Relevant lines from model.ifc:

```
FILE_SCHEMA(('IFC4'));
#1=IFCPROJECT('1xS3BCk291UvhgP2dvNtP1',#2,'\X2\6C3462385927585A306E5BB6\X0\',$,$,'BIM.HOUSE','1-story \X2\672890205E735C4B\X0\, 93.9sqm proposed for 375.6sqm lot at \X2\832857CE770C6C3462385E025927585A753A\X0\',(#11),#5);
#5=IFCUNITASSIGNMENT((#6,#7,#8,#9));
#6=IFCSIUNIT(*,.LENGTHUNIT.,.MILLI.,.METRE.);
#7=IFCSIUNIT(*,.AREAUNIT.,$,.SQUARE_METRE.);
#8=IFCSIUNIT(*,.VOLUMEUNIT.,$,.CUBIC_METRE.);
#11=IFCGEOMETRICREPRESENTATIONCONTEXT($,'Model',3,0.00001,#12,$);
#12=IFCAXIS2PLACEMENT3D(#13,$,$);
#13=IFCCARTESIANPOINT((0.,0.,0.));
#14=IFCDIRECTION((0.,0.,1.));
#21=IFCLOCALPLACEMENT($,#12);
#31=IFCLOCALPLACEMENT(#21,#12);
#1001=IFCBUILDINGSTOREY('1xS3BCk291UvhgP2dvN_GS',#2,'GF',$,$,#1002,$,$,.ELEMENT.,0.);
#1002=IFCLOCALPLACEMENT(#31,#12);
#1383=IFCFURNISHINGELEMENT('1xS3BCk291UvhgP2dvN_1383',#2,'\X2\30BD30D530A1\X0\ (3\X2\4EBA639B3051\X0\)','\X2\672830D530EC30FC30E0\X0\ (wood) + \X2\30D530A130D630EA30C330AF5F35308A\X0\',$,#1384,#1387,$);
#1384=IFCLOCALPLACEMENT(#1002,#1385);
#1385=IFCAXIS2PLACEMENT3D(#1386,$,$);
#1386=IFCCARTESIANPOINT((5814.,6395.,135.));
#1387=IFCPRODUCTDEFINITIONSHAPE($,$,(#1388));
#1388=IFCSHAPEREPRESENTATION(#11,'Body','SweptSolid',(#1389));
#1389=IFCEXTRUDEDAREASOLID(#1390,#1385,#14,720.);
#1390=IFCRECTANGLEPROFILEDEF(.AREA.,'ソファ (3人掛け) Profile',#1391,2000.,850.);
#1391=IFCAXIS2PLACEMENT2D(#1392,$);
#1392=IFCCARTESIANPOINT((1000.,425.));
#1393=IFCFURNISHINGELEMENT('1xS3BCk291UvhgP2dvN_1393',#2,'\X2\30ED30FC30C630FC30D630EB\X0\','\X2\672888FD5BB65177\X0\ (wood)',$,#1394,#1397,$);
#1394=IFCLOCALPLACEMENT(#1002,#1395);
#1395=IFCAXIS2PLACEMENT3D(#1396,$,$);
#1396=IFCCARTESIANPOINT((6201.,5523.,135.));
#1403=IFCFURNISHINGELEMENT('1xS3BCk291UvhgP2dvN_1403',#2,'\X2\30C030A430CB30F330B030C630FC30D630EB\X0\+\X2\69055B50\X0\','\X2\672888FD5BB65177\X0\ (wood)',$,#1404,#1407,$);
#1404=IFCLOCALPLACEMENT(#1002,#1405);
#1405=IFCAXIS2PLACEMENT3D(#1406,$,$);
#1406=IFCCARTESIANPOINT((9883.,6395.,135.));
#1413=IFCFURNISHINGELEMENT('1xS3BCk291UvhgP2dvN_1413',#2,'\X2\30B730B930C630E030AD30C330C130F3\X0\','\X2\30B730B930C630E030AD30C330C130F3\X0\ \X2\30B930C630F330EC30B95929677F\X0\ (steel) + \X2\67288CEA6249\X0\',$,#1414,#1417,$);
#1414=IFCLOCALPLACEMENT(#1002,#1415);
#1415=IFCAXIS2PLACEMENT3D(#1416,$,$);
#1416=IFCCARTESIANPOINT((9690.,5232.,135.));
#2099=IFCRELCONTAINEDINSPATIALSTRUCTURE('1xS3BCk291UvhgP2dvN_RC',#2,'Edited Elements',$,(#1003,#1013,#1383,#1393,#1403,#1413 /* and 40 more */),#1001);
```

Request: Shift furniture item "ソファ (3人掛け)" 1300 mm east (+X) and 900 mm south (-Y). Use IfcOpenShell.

```python
import ifcopenshell
import ifcopenshell.api.geometry
import ifcopenshell.util.placement
import ifcopenshell.util.unit

model = ifcopenshell.open("model.ifc")
unit_scale = ifcopenshell.util.unit.calculate_unit_scale(model)

item = model.by_guid("1xS3BCk291UvhgP2dvN_1383")
matrix = ifcopenshell.util.placement.get_local_placement(item.ObjectPlacement)
matrix[0, 3] += 1.3 / unit_scale
matrix[1, 3] -= 0.9 / unit_scale
ifcopenshell.api.geometry.edit_object_placement(model, product=item, matrix=matrix, is_si=False)

print(ifcopenshell.util.placement.get_local_placement(item.ObjectPlacement).round(3) + 0.0)

model.write("model_rev.ifc")
```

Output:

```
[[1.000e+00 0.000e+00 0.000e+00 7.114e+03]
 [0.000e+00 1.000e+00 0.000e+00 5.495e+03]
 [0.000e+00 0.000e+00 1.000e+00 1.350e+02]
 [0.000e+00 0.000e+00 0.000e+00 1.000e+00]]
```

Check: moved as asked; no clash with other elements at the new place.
